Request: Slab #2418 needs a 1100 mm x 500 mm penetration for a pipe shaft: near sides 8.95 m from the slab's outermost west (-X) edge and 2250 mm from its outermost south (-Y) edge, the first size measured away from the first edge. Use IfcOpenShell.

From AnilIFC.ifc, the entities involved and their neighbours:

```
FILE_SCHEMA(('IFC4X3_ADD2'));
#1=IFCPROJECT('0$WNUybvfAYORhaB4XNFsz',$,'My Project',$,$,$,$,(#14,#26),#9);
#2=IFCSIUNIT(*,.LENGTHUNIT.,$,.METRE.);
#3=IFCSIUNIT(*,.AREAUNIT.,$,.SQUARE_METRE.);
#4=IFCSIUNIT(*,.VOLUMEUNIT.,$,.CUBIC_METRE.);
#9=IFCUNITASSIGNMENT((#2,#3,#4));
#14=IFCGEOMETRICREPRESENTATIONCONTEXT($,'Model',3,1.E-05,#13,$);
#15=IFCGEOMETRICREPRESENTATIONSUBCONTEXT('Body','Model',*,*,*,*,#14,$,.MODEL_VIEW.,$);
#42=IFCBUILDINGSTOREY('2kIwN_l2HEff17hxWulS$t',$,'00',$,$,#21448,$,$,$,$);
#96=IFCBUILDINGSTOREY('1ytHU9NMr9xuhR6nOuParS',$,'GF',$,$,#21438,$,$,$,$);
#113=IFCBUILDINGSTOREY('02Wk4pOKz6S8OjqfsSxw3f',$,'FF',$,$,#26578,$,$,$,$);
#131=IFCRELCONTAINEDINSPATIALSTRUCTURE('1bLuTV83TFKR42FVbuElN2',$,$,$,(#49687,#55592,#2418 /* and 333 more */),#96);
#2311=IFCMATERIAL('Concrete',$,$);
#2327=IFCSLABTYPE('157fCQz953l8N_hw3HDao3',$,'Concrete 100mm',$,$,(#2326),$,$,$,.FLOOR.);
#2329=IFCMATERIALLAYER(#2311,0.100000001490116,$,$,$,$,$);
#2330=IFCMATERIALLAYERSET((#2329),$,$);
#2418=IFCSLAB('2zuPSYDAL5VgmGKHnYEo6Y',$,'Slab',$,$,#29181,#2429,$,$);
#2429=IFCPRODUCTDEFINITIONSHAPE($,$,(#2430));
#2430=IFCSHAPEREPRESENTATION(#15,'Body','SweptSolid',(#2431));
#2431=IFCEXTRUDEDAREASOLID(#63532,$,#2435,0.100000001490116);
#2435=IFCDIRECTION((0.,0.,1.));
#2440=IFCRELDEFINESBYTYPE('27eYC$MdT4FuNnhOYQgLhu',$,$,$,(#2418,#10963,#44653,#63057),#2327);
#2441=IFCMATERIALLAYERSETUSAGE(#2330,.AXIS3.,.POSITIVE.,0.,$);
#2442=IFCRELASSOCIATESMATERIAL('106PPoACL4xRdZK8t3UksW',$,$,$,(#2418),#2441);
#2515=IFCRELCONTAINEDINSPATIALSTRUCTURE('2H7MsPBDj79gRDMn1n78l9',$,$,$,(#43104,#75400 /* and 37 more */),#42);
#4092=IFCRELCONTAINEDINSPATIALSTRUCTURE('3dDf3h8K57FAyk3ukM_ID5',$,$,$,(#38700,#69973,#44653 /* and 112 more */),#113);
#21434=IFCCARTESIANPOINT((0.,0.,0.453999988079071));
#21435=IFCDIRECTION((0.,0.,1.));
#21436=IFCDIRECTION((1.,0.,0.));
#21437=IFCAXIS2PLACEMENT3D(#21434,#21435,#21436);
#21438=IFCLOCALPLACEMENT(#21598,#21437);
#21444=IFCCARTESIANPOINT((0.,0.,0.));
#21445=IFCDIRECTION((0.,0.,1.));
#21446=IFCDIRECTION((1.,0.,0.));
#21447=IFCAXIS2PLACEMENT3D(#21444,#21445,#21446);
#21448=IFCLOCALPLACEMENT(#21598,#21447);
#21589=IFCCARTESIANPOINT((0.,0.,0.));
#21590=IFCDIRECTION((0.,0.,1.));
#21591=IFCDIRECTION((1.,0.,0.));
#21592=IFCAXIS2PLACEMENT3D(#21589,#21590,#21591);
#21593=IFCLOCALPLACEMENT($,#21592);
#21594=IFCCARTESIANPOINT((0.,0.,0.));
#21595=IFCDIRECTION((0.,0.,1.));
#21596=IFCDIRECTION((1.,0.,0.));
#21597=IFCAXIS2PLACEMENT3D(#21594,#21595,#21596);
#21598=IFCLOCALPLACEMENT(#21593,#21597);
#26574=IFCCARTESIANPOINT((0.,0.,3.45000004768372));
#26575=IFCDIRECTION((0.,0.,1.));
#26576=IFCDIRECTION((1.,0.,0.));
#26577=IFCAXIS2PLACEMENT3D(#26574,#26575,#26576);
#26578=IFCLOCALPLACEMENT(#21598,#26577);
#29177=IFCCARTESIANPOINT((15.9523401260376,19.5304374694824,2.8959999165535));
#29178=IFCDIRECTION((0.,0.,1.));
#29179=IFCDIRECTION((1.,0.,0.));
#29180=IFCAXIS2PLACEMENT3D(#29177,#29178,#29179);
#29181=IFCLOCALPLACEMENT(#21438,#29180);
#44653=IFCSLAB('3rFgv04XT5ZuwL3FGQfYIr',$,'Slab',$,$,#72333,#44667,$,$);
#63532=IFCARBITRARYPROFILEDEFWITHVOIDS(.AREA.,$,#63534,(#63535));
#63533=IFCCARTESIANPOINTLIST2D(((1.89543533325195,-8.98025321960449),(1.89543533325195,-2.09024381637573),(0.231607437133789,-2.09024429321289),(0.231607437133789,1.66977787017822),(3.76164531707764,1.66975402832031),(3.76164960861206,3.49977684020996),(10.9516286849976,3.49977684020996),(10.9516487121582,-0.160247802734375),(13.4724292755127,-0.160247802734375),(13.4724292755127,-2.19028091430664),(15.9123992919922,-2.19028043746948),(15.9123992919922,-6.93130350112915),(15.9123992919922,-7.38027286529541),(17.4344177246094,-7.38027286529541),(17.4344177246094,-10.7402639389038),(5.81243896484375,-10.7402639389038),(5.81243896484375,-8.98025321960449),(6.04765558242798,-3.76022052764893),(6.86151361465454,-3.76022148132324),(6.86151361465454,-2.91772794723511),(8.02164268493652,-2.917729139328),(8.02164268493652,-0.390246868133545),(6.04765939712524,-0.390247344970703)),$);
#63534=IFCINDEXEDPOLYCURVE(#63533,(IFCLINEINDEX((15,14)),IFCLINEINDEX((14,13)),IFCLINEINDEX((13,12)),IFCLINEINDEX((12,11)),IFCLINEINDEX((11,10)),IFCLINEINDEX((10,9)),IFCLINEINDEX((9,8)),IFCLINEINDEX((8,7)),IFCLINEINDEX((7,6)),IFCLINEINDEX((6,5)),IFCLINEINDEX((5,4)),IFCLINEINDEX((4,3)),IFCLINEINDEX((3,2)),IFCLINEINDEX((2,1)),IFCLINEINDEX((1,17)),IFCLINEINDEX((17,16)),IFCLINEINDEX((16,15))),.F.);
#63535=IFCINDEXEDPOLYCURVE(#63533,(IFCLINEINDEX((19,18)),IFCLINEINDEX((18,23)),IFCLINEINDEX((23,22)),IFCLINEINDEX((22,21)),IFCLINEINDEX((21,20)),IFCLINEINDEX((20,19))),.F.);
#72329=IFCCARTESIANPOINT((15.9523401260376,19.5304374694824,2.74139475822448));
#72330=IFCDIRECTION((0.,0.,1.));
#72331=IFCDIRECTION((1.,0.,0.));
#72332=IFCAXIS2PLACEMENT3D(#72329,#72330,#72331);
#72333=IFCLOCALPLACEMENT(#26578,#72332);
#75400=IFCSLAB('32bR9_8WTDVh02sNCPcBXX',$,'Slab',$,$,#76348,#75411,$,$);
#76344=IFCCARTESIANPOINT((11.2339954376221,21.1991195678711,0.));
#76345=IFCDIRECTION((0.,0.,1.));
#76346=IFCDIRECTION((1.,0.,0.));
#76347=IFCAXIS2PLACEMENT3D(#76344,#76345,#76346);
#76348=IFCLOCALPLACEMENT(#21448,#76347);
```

```python
import numpy as np
import ifcopenshell
import ifcopenshell.api.feature
import ifcopenshell.api.geometry
import ifcopenshell.api.root
import ifcopenshell.geom
import ifcopenshell.util.placement
import ifcopenshell.util.representation
import ifcopenshell.util.shape
import ifcopenshell.util.unit

model = ifcopenshell.open("AnilIFC.ifc")
unit_scale = ifcopenshell.util.unit.calculate_unit_scale(model)
settings = ifcopenshell.geom.settings()


def volume(element):
    """Net volume in cubic metres, openings subtracted."""
    shape = ifcopenshell.geom.create_shape(settings, element)
    return ifcopenshell.util.shape.get_volume(shape.geometry)


slab = model.by_guid("2zuPSYDAL5VgmGKHnYEo6Y")
before = volume(slab)

# Extent in the slab's own axes, in metres. The edges named are its -X and -Y sides.
slab_shape = ifcopenshell.geom.create_shape(settings, slab)
vertices = ifcopenshell.util.shape.get_vertices(slab_shape.geometry)
x_min, y_min, bottom = vertices.min(axis=0)
top = vertices[:, 2].max()

opening = ifcopenshell.api.root.create_entity(model, ifc_class="IfcOpeningElement", name="Pipe shaft opening", predefined_type="OPENING")
context = ifcopenshell.util.representation.get_context(model, "Model", "Body", "MODEL_VIEW")
width, depth = 1.1, 0.5
outline = [(0.0, 0.0), (width, 0.0), (width, depth), (0.0, depth), (0.0, 0.0)]
# Overshoot both faces by 50 mm so the cut is clean.
shape = ifcopenshell.api.geometry.add_slab_representation(
    model, context=context, depth=top - bottom + 0.1, polyline=outline
)
ifcopenshell.api.geometry.assign_representation(model, product=opening, representation=shape)

matrix = ifcopenshell.util.placement.get_local_placement(slab.ObjectPlacement)
matrix[:, 3] = matrix @ np.append(np.array([x_min + 8.95, y_min + 2.25, bottom - 0.05]) / unit_scale, 1.0)
ifcopenshell.api.geometry.edit_object_placement(model, product=opening, matrix=matrix, is_si=False)
ifcopenshell.api.feature.add_feature(model, feature=opening, element=slab)

after = volume(slab)

print(f"slab volume {before:.3f} -> {after:.3f} m3")

model.write("AnilIFC_updated.ifc")
```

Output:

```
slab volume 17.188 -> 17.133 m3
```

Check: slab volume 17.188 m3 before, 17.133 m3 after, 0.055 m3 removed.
